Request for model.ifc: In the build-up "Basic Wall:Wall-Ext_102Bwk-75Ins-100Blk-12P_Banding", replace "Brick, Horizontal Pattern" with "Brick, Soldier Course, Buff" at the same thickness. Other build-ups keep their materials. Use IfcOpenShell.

First a look at what the model holds.

```python
import ifcopenshell
import ifcopenshell.util.element

model = ifcopenshell.open("model.ifc")
print(model.schema)
for layer_set in model.by_type("IfcMaterialLayerSet"):
    if layer_set.LayerSetName == "Basic Wall:Wall-Ext_102Bwk-75Ins-100Blk-12P_Banding":
        for layer in layer_set.MaterialLayers:
            print(layer.id(), layer.Material and layer.Material.Name, layer.LayerThickness, sep=" | ")
        print(len(ifcopenshell.util.element.get_elements_by_material(model, layer_set)), "elements and types use it")
print(sorted(m.Name for m in model.by_type("IfcMaterial") if m.Name)[:60])
```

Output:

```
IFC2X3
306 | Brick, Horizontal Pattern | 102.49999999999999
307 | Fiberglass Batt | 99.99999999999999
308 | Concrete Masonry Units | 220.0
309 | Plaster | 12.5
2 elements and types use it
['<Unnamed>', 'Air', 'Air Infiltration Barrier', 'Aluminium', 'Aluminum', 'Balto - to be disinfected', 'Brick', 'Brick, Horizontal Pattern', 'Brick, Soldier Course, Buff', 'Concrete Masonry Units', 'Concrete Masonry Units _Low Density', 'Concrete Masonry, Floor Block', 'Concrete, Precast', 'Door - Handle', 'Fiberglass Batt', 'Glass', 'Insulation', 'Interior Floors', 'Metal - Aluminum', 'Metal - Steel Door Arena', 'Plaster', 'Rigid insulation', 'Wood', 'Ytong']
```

```python
import ifcopenshell
import ifcopenshell.api.material

model = ifcopenshell.open("model.ifc")

layer_set = next(s for s in model.by_type("IfcMaterialLayerSet") if s.LayerSetName == "Basic Wall:Wall-Ext_102Bwk-75Ins-100Blk-12P_Banding")
layer = next(l for l in layer_set.MaterialLayers if l.Material and l.Material.Name == "Brick, Horizontal Pattern")
material = next(m for m in model.by_type("IfcMaterial") if m.Name == "Brick, Soldier Course, Buff")

# Point this one layer at the other material; renaming the old one would change it everywhere.
ifcopenshell.api.material.edit_layer(model, layer=layer, attributes={}, material=material)

print([l.Material.Name if l.Material else None for l in layer_set.MaterialLayers])

model.write("model_updated.ifc")
```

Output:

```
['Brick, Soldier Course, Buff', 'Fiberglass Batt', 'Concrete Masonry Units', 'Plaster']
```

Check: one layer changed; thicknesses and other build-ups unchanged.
